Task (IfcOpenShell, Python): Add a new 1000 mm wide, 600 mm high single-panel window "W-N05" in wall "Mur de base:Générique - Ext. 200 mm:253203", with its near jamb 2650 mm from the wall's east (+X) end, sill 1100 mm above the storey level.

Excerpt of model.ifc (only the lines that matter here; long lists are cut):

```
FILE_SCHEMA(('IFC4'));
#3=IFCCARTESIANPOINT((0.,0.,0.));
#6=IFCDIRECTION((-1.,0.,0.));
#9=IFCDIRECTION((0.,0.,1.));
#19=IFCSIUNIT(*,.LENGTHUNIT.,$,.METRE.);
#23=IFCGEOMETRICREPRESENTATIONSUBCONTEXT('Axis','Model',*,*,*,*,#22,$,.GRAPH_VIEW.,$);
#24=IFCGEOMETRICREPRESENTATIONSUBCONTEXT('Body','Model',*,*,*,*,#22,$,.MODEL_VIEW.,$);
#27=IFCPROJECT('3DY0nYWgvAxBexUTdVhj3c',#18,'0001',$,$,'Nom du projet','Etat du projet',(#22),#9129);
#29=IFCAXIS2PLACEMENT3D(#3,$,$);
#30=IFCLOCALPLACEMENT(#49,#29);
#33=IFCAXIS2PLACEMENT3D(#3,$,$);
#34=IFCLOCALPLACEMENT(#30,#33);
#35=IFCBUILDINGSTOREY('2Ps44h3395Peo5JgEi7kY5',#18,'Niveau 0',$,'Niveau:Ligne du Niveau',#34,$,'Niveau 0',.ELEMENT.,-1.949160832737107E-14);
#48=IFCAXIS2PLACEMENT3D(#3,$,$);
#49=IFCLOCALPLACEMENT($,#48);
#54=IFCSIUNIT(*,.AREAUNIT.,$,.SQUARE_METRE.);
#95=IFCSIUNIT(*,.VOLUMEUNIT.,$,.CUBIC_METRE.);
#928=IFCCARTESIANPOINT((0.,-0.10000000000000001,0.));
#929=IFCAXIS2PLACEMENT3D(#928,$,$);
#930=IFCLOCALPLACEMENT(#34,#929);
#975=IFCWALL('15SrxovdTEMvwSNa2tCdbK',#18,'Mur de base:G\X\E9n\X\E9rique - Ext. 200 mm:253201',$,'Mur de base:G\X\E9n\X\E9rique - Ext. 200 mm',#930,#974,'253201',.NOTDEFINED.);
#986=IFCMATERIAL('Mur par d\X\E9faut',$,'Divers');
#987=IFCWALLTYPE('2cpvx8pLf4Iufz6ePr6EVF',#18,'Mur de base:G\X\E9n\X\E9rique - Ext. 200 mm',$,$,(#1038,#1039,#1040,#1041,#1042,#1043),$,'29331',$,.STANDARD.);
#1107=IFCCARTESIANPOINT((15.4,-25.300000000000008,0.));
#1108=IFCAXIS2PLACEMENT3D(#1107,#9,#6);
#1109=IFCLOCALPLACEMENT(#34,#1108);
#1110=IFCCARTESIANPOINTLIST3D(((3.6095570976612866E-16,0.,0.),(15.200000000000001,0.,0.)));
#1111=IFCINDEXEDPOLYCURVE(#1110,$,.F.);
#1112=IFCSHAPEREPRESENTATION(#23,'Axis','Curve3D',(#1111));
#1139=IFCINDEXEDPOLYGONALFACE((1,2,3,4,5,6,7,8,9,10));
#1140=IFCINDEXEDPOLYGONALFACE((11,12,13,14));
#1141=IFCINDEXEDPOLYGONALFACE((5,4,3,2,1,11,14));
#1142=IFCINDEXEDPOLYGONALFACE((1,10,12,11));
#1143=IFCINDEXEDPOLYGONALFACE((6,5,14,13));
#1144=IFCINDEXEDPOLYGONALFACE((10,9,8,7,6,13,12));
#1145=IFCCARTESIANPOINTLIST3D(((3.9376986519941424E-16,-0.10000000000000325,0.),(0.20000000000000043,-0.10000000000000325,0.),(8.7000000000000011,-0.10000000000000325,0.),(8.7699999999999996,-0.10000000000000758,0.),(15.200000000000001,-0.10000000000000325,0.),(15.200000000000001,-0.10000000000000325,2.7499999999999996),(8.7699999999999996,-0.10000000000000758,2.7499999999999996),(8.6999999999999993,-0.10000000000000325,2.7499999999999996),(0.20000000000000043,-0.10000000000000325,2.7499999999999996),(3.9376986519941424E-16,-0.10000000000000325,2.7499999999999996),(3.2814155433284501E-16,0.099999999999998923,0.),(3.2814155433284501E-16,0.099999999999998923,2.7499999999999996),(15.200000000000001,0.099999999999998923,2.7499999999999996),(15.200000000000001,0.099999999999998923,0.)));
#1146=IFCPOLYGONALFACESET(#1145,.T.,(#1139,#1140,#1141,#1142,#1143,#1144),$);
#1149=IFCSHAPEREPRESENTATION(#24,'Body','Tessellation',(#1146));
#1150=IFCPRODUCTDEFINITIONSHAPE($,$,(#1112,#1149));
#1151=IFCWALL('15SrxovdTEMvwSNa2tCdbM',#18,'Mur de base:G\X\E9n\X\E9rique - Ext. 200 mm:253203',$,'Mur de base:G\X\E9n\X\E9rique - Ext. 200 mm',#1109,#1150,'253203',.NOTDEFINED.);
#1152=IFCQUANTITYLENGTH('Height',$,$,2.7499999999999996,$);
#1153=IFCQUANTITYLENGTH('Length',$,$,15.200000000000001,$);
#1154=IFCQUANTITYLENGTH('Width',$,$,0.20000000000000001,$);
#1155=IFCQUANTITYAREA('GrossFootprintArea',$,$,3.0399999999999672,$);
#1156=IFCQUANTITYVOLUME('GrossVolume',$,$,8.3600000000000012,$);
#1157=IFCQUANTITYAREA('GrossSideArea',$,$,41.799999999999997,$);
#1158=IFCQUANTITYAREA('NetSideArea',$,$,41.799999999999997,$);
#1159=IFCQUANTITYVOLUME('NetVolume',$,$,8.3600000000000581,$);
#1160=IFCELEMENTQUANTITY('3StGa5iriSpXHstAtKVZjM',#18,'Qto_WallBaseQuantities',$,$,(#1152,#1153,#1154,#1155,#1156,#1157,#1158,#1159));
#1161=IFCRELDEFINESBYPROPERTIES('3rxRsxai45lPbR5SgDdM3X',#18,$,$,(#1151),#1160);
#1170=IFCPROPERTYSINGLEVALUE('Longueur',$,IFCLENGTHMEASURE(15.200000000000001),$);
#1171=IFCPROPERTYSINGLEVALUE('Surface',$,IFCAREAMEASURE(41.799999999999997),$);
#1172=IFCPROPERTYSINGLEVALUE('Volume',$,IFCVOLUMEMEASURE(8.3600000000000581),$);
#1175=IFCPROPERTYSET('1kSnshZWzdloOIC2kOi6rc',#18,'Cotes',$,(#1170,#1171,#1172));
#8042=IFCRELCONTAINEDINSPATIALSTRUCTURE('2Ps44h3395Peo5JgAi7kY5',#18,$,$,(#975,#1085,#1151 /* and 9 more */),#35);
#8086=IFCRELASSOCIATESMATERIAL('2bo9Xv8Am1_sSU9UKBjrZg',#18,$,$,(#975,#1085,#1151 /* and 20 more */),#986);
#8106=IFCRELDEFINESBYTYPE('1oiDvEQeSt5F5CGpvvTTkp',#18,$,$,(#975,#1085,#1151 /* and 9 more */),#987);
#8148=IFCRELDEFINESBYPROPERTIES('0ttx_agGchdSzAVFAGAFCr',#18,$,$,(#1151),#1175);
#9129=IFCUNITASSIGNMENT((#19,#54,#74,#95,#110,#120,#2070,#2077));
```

```python
import numpy as np
import ifcopenshell
import ifcopenshell.api.feature
import ifcopenshell.api.geometry
import ifcopenshell.api.pset
import ifcopenshell.api.root
import ifcopenshell.api.spatial
import ifcopenshell.geom
import ifcopenshell.util.element
import ifcopenshell.util.placement
import ifcopenshell.util.representation
import ifcopenshell.util.shape
import ifcopenshell.util.unit

model = ifcopenshell.open("model.ifc")
unit_scale = ifcopenshell.util.unit.calculate_unit_scale(model)
area_scale = ifcopenshell.util.unit.calculate_unit_scale(model, "AREAUNIT")
volume_scale = ifcopenshell.util.unit.calculate_unit_scale(model, "VOLUMEUNIT")
settings = ifcopenshell.geom.settings()


def volume(element):
    """Net volume in cubic metres, openings subtracted."""
    shape = ifcopenshell.geom.create_shape(settings, element)
    return ifcopenshell.util.shape.get_volume(shape.geometry)


wall = model.by_id(1151)
storey = ifcopenshell.util.element.get_container(wall, ifc_class="IfcBuildingStorey")
context = ifcopenshell.util.representation.get_context(model, "Model", "Body", "MODEL_VIEW")
before = volume(wall)

width, height, from_end, sill = 1, 0.6, 2.65, 1.1  # metres

# The wall runs along its own X axis, and the end named is its -X end.
wall_shape = ifcopenshell.geom.create_shape(settings, wall)
x, y, z = ifcopenshell.util.shape.get_vertices(wall_shape.geometry).T
start = x.min() + from_end
face, thickness = float(y.min()), float(y.max() - y.min())
wall_matrix = ifcopenshell.util.placement.get_local_placement(wall.ObjectPlacement)
level = ifcopenshell.util.placement.get_local_placement(storey.ObjectPlacement)[2, 3]


def in_wall(x, y):
    """Placement at x, y metres in the wall's axes, at sill height."""
    matrix = wall_matrix.copy()
    matrix[:, 3] = wall_matrix @ np.array([x / unit_scale, y / unit_scale, 0.0, 1.0])
    matrix[2, 3] = level + sill / unit_scale
    return matrix


# Opening: a box that overshoots both wall faces by 50 mm.
opening = ifcopenshell.api.root.create_entity(model, ifc_class="IfcOpeningElement", predefined_type="OPENING")
box = ifcopenshell.api.geometry.add_wall_representation(
    model, context=context, length=width, height=height, thickness=thickness + 0.1
)
ifcopenshell.api.geometry.assign_representation(model, product=opening, representation=box)
ifcopenshell.api.geometry.edit_object_placement(model, product=opening, matrix=in_wall(start, face - 0.05), is_si=False)
ifcopenshell.api.feature.add_feature(model, feature=opening, element=wall)

window = ifcopenshell.api.root.create_entity(model, ifc_class="IfcWindow", name="W-N05", predefined_type="WINDOW")
window.OverallWidth, window.OverallHeight = width / unit_scale, height / unit_scale
window.PartitioningType = "SINGLE_PANEL"
body = ifcopenshell.api.geometry.add_window_representation(
    model,
    context=context,
    overall_width=window.OverallWidth,
    overall_height=window.OverallHeight,
    partition_type="SINGLE_PANEL",
)
ifcopenshell.api.geometry.assign_representation(model, product=window, representation=body)
ifcopenshell.api.spatial.assign_container(model, products=[window], relating_structure=storey)
ifcopenshell.api.feature.add_filling(model, opening=opening, element=window)

# Centre the window in the wall's thickness.
ifcopenshell.api.geometry.edit_object_placement(model, product=window, matrix=in_wall(start, face), is_si=False)
window_shape = ifcopenshell.geom.create_shape(settings, window)
depth = ifcopenshell.util.shape.get_vertices(window_shape.geometry)[:, 1]
offset = face + thickness / 2 - (depth.min() + depth.max()) / 2
ifcopenshell.api.geometry.edit_object_placement(model, product=window, matrix=in_wall(start, offset), is_si=False)

after = volume(wall)

# Update the wall's stored quantities.
qto = model.by_id(ifcopenshell.util.element.get_pset(wall, "Qto_WallBaseQuantities", should_inherit=False)["id"])
ifcopenshell.api.pset.edit_qto(model, qto=qto, properties={
    "NetSideArea": after / thickness / area_scale,
    "NetVolume": after / volume_scale,
})
pset = model.by_id(ifcopenshell.util.element.get_pset(wall, "Cotes", should_inherit=False)["id"])
ifcopenshell.api.pset.edit_pset(model, pset=pset, properties={
    "Surface": model.create_entity("IfcAreaMeasure", after / thickness / area_scale),
    "Volume": model.create_entity("IfcVolumeMeasure", after / volume_scale),
})

print(f"wall volume {before:.3f} -> {after:.3f} m3")

model.write("model_edited.ifc")
```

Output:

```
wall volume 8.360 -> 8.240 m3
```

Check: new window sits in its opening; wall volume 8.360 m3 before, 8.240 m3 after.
